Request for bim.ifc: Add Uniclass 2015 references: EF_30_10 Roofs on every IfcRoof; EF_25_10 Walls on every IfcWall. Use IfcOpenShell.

First a look at what the model holds.

```python
import ifcopenshell

model = ifcopenshell.open("bim.ifc")
print(model.schema)
print("classifications:", [c.Name for c in model.by_type("IfcClassification")])
for ifc_class in ("IfcDoor", "IfcRoof", "IfcStair", "IfcWall", "IfcWindow"):
    print(ifc_class, len(model.by_type(ifc_class)))
```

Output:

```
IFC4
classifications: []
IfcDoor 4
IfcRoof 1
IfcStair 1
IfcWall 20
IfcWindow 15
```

```python
import ifcopenshell
import ifcopenshell.api.classification

model = ifcopenshell.open("bim.ifc")

system = ifcopenshell.api.classification.add_classification(model, classification="Uniclass 2015")

codes = {
    "IfcRoof": ("EF_30_10", "Roofs"),
    "IfcWall": ("EF_25_10", "Walls"),
}
for ifc_class, (code, name) in codes.items():
    products = model.by_type(ifc_class)
    ifcopenshell.api.classification.add_reference(
        model, products=products, classification=system, identification=code, name=name
    )
    print(code, len(products))

model.write("bim_updated.ifc")
```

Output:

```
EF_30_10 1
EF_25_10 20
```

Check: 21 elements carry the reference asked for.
